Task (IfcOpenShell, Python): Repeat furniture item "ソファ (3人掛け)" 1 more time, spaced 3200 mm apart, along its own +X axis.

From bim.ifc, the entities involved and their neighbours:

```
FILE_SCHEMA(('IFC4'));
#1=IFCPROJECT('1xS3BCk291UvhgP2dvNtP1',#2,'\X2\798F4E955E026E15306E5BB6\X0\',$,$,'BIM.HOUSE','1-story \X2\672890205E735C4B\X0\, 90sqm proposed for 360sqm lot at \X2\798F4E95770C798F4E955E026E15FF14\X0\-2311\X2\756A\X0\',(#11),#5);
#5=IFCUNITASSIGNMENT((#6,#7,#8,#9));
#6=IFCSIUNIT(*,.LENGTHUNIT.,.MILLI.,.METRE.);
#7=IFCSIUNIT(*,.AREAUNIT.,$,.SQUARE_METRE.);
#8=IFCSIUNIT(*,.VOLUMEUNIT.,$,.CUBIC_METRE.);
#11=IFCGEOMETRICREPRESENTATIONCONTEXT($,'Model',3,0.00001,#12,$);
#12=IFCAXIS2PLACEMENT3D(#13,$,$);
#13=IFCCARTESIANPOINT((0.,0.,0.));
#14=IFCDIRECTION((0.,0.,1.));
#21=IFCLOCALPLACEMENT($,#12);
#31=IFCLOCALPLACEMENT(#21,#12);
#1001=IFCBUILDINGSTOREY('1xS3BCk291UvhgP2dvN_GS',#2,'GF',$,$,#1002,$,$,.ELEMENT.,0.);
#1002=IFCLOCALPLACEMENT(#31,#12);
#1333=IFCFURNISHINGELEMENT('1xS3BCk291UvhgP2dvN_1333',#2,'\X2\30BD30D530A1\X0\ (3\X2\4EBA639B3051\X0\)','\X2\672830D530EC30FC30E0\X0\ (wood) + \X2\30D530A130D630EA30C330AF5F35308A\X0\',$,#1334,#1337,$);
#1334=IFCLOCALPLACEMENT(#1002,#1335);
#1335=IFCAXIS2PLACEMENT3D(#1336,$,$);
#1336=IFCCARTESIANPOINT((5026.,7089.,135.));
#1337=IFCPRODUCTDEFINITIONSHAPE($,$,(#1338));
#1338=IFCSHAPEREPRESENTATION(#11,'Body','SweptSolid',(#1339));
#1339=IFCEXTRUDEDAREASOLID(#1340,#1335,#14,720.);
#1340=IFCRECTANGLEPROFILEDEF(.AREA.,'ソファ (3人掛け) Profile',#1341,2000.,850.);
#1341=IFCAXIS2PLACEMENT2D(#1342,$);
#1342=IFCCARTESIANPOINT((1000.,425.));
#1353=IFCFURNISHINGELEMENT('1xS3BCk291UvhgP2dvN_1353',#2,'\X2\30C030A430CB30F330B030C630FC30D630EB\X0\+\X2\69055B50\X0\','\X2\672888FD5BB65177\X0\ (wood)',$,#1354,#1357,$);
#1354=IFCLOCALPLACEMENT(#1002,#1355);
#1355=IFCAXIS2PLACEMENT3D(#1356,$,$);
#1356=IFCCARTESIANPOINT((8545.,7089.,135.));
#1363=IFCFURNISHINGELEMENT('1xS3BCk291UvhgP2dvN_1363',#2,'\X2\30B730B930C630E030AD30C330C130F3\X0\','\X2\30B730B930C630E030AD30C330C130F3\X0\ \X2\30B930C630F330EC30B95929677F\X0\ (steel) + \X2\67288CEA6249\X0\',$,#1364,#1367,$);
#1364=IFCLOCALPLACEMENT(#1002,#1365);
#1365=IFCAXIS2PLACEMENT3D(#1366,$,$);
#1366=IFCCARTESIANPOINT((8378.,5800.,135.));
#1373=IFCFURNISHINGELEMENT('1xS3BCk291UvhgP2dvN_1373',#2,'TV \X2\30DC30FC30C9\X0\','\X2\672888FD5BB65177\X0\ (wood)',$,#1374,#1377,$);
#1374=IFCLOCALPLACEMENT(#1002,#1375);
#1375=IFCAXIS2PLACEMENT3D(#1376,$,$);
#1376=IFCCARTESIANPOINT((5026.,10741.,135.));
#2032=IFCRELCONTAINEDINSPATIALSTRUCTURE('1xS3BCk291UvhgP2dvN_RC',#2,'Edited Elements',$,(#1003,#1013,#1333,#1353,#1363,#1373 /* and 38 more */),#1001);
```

```python
import ifcopenshell
import ifcopenshell.api.geometry
import ifcopenshell.api.root
import ifcopenshell.util.element
import ifcopenshell.util.placement
import ifcopenshell.util.unit

model = ifcopenshell.open("bim.ifc")
unit_scale = ifcopenshell.util.unit.calculate_unit_scale(model)


def reuse_history(source, copy):
    """copy_class also copies each property set's owner history, people and application; keep the originals."""
    for rel in copy.IsDefinedBy:
        if rel.is_a("IfcRelDefinesByProperties") and (history := rel.RelatingPropertyDefinition.OwnerHistory):
            rel.RelatingPropertyDefinition.OwnerHistory = source.OwnerHistory
            ifcopenshell.util.element.remove_deep2(model, history)


source = model.by_guid("1xS3BCk291UvhgP2dvN_1333")
base = ifcopenshell.util.placement.get_local_placement(source.ObjectPlacement)
step = base[:3, 0] * 3.2 / unit_scale

for i in range(1, 2):
    copy = ifcopenshell.api.root.copy_class(model, product=source)
    copy.Representation = ifcopenshell.util.element.copy_deep(
        model, source.Representation, exclude=["IfcGeometricRepresentationContext", "IfcRepresentationMap"]
    )
    reuse_history(source, copy)
    matrix = base.copy()
    matrix[:3, 3] += i * step
    print("added at", matrix[:3, 3].round(3) + 0.0)
    ifcopenshell.api.geometry.edit_object_placement(model, product=copy, matrix=matrix, is_si=False)

model.write("bim-out.ifc")
```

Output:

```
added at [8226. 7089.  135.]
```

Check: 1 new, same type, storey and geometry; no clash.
